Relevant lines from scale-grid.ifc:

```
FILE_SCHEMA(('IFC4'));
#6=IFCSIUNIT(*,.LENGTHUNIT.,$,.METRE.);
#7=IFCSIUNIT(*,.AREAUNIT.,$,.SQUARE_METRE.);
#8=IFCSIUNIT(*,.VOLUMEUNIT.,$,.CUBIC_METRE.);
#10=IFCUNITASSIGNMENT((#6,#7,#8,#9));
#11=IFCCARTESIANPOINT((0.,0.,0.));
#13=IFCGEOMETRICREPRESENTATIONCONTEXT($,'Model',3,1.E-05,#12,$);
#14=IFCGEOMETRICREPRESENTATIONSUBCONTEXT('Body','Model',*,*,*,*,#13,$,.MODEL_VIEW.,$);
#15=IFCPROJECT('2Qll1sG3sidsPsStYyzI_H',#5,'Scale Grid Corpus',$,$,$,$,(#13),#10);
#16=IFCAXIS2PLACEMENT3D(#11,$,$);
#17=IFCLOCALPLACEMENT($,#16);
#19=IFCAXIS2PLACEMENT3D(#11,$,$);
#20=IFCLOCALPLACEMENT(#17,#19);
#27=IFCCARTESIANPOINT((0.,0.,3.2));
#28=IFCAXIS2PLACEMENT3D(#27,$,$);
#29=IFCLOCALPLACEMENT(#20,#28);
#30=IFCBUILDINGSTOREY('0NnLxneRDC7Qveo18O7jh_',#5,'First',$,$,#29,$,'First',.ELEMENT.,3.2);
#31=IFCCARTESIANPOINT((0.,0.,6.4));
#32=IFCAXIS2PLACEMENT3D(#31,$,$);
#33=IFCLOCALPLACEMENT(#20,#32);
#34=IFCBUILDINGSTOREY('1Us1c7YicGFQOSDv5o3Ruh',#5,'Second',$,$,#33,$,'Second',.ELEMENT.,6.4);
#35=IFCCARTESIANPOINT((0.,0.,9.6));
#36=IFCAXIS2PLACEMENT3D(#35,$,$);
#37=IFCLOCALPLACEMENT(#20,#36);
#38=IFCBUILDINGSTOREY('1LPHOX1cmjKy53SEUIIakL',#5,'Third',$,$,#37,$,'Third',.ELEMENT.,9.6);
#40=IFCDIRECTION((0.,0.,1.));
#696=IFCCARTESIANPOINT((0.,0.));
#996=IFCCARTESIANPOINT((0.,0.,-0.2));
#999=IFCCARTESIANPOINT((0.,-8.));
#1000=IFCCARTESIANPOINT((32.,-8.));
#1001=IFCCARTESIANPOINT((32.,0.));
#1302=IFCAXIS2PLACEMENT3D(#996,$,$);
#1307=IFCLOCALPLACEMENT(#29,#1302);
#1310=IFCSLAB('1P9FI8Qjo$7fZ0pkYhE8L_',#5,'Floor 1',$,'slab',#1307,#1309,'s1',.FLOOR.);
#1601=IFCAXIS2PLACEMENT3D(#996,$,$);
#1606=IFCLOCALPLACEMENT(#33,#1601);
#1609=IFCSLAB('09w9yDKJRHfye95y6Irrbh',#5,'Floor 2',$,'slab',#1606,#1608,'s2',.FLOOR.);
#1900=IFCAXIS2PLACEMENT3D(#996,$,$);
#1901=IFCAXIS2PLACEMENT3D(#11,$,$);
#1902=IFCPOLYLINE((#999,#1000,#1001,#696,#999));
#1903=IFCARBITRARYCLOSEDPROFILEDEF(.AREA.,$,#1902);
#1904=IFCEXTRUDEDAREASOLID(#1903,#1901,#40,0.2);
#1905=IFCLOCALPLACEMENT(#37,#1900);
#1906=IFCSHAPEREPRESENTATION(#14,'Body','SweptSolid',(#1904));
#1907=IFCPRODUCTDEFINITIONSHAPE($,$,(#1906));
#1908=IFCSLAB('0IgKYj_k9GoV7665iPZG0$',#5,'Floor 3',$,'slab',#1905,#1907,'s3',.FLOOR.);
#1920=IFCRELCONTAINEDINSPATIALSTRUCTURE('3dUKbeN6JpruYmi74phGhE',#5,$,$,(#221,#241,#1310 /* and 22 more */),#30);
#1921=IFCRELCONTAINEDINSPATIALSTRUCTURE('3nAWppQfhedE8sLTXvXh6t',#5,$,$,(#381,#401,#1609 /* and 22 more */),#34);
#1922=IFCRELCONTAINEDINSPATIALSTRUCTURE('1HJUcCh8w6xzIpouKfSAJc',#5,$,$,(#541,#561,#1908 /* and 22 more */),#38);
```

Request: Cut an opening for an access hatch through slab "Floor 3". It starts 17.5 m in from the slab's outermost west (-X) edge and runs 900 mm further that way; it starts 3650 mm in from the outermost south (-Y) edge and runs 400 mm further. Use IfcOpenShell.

```python
import numpy as np
import ifcopenshell
import ifcopenshell.api.feature
import ifcopenshell.api.geometry
import ifcopenshell.api.root
import ifcopenshell.geom
import ifcopenshell.util.placement
import ifcopenshell.util.representation
import ifcopenshell.util.shape
import ifcopenshell.util.unit

model = ifcopenshell.open("scale-grid.ifc")
unit_scale = ifcopenshell.util.unit.calculate_unit_scale(model)
settings = ifcopenshell.geom.settings()


def volume(element):
    """Net volume in cubic metres, openings subtracted."""
    shape = ifcopenshell.geom.create_shape(settings, element)
    return ifcopenshell.util.shape.get_volume(shape.geometry)


slab = model.by_id(1908)
before = volume(slab)

# Extent in the slab's own axes, in metres. The edges named are its -X and -Y sides.
slab_shape = ifcopenshell.geom.create_shape(settings, slab)
vertices = ifcopenshell.util.shape.get_vertices(slab_shape.geometry)
x_min, y_min, bottom = vertices.min(axis=0)
top = vertices[:, 2].max()

opening = ifcopenshell.api.root.create_entity(model, ifc_class="IfcOpeningElement", name="Access hatch opening", predefined_type="OPENING")
context = ifcopenshell.util.representation.get_context(model, "Model", "Body", "MODEL_VIEW")
width, depth = 0.9, 0.4
outline = [(0.0, 0.0), (width, 0.0), (width, depth), (0.0, depth), (0.0, 0.0)]
# Overshoot both faces by 50 mm so the cut is clean.
shape = ifcopenshell.api.geometry.add_slab_representation(
    model, context=context, depth=top - bottom + 0.1, polyline=outline
)
ifcopenshell.api.geometry.assign_representation(model, product=opening, representation=shape)

matrix = ifcopenshell.util.placement.get_local_placement(slab.ObjectPlacement)
matrix[:, 3] = matrix @ np.append(np.array([x_min + 17.5, y_min + 3.65, bottom - 0.05]) / unit_scale, 1.0)
ifcopenshell.api.geometry.edit_object_placement(model, product=opening, matrix=matrix, is_si=False)
ifcopenshell.api.feature.add_feature(model, feature=opening, element=slab)

after = volume(slab)

print(f"slab volume {before:.3f} -> {after:.3f} m3")

model.write("scale-grid_edited.ifc")
```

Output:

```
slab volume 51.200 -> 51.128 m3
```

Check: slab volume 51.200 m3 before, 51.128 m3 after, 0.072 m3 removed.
